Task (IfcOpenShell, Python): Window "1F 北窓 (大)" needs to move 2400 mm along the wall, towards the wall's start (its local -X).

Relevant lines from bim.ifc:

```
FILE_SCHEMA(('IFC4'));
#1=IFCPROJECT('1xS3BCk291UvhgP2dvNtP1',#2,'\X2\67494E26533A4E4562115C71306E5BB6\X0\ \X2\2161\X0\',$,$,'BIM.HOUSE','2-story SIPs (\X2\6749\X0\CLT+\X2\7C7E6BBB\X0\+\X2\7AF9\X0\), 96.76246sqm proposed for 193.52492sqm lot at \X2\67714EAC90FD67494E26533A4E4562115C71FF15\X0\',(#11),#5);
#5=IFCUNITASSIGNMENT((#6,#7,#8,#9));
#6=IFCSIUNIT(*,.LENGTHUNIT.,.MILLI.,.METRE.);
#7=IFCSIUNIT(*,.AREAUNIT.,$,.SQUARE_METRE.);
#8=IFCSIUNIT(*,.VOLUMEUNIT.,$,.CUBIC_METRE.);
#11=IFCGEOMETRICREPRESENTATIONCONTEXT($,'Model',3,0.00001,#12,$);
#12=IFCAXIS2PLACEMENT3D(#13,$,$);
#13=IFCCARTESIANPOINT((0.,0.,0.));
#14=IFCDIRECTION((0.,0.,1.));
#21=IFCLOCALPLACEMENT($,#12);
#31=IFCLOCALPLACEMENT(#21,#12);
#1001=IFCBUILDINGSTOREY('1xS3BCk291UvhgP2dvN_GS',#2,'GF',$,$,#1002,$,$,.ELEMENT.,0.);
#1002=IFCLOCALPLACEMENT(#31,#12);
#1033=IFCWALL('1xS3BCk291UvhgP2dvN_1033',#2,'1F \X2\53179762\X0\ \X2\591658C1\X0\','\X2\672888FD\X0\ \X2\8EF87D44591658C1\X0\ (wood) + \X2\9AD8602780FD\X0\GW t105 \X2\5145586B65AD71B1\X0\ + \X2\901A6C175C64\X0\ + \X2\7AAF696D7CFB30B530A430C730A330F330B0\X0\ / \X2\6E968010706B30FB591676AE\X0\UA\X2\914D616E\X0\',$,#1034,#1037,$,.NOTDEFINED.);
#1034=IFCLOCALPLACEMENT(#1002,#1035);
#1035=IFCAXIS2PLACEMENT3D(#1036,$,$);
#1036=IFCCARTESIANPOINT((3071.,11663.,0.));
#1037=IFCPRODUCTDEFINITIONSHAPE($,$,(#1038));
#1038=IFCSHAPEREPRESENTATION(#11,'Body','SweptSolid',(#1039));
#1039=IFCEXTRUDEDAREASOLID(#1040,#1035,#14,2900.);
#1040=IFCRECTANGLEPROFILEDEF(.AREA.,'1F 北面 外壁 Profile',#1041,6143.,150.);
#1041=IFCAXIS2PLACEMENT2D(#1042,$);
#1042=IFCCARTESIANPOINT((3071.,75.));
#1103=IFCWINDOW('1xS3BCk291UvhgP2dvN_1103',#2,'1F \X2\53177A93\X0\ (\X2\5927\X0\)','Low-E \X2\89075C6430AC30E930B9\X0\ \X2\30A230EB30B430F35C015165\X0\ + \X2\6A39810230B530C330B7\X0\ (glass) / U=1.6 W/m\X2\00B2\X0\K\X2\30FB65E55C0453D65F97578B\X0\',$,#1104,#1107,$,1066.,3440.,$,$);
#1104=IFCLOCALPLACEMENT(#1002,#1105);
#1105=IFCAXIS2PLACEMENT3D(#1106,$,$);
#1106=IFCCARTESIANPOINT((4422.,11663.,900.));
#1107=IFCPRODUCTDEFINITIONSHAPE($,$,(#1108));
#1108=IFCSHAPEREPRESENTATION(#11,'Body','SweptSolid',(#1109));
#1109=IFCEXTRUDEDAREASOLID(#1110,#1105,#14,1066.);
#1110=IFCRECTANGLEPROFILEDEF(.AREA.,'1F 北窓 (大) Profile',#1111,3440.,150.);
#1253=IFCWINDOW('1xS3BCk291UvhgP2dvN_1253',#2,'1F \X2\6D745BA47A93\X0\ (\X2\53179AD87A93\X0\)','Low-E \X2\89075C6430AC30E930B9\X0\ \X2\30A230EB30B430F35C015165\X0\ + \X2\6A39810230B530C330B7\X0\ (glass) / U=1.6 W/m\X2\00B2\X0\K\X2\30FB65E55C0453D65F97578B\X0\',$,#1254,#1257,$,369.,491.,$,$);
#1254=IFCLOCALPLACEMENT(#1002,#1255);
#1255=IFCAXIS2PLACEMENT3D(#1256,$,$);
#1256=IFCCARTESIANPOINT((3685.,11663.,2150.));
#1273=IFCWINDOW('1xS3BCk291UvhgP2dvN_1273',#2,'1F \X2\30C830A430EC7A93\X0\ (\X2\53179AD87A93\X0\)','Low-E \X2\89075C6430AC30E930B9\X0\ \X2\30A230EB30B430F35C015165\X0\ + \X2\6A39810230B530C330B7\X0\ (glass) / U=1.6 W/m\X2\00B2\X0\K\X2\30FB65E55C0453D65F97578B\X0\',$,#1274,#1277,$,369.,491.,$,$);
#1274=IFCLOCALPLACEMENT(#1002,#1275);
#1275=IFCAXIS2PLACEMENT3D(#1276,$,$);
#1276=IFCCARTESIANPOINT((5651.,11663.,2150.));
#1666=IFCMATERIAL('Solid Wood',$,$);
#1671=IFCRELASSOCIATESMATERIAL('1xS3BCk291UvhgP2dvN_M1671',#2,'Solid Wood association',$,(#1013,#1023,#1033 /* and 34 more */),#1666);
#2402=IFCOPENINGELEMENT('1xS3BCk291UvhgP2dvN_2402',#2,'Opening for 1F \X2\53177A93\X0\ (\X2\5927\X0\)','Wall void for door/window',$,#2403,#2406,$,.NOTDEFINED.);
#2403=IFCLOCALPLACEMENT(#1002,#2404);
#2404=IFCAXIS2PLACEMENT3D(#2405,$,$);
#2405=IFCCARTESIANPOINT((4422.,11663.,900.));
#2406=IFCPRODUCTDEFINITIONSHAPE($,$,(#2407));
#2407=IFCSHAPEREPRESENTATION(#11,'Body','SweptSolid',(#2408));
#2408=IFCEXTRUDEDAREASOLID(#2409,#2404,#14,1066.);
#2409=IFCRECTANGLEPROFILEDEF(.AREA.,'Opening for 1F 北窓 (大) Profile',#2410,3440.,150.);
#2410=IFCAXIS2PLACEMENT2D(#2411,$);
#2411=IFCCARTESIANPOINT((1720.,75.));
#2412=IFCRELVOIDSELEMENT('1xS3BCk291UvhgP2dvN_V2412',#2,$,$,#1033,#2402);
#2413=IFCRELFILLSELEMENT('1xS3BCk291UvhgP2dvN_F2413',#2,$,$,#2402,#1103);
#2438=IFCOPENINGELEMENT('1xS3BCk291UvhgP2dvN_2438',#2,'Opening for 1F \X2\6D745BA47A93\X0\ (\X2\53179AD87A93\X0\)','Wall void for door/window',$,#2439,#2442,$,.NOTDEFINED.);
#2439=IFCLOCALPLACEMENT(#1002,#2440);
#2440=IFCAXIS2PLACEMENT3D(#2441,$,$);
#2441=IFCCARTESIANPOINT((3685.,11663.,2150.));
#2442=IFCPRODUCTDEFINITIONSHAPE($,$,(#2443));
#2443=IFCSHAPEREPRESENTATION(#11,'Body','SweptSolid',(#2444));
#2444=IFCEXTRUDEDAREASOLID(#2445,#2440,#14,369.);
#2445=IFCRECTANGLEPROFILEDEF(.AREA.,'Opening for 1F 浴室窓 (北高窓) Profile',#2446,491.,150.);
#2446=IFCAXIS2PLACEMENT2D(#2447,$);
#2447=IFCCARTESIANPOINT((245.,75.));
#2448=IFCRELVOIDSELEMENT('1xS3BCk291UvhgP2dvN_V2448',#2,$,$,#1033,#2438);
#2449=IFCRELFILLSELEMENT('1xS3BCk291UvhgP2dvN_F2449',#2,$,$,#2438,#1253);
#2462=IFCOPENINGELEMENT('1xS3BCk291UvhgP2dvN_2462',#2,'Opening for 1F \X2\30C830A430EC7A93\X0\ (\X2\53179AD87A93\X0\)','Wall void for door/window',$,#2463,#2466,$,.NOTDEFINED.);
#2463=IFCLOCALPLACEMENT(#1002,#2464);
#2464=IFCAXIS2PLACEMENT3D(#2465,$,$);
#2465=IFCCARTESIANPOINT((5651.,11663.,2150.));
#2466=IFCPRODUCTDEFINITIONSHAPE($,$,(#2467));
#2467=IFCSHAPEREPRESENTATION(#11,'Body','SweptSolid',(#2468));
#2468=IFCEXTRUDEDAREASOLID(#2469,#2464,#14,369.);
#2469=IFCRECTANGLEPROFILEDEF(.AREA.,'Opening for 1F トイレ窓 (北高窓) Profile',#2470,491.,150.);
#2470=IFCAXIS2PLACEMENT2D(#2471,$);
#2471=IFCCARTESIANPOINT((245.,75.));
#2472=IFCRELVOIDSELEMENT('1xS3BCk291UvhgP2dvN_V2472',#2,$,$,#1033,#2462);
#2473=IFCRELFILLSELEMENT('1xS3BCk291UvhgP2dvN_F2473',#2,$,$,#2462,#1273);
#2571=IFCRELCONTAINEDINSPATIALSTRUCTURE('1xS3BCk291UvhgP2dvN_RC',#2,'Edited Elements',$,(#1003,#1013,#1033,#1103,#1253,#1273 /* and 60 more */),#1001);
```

```python
import ifcopenshell
import ifcopenshell.api.geometry
import ifcopenshell.util.placement
import ifcopenshell.util.unit

model = ifcopenshell.open("bim.ifc")
unit_scale = ifcopenshell.util.unit.calculate_unit_scale(model)

window = model.by_guid("1xS3BCk291UvhgP2dvN_1103")
opening = window.FillsVoids[0].RelatingOpeningElement
wall = opening.VoidsElements[0].RelatingBuildingElement

wall_matrix = ifcopenshell.util.placement.get_local_placement(wall.ObjectPlacement)
shift = wall_matrix[:3, 0] * -2.4 / unit_scale
before = ifcopenshell.util.placement.get_local_placement(window.ObjectPlacement)[:3, 3].copy()

# The window is not placed relative to its opening, so move both.
for product in (opening, window):
    matrix = ifcopenshell.util.placement.get_local_placement(product.ObjectPlacement)
    matrix[:3, 3] += shift
    ifcopenshell.api.geometry.edit_object_placement(model, product=product, matrix=matrix, is_si=False)

after = ifcopenshell.util.placement.get_local_placement(window.ObjectPlacement)[:3, 3]
print("window moved by", (after - before).round(3) + 0.0)

model.write("bim_updated.ifc")
```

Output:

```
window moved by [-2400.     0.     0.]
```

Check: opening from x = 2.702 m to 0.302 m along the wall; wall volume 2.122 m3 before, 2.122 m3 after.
